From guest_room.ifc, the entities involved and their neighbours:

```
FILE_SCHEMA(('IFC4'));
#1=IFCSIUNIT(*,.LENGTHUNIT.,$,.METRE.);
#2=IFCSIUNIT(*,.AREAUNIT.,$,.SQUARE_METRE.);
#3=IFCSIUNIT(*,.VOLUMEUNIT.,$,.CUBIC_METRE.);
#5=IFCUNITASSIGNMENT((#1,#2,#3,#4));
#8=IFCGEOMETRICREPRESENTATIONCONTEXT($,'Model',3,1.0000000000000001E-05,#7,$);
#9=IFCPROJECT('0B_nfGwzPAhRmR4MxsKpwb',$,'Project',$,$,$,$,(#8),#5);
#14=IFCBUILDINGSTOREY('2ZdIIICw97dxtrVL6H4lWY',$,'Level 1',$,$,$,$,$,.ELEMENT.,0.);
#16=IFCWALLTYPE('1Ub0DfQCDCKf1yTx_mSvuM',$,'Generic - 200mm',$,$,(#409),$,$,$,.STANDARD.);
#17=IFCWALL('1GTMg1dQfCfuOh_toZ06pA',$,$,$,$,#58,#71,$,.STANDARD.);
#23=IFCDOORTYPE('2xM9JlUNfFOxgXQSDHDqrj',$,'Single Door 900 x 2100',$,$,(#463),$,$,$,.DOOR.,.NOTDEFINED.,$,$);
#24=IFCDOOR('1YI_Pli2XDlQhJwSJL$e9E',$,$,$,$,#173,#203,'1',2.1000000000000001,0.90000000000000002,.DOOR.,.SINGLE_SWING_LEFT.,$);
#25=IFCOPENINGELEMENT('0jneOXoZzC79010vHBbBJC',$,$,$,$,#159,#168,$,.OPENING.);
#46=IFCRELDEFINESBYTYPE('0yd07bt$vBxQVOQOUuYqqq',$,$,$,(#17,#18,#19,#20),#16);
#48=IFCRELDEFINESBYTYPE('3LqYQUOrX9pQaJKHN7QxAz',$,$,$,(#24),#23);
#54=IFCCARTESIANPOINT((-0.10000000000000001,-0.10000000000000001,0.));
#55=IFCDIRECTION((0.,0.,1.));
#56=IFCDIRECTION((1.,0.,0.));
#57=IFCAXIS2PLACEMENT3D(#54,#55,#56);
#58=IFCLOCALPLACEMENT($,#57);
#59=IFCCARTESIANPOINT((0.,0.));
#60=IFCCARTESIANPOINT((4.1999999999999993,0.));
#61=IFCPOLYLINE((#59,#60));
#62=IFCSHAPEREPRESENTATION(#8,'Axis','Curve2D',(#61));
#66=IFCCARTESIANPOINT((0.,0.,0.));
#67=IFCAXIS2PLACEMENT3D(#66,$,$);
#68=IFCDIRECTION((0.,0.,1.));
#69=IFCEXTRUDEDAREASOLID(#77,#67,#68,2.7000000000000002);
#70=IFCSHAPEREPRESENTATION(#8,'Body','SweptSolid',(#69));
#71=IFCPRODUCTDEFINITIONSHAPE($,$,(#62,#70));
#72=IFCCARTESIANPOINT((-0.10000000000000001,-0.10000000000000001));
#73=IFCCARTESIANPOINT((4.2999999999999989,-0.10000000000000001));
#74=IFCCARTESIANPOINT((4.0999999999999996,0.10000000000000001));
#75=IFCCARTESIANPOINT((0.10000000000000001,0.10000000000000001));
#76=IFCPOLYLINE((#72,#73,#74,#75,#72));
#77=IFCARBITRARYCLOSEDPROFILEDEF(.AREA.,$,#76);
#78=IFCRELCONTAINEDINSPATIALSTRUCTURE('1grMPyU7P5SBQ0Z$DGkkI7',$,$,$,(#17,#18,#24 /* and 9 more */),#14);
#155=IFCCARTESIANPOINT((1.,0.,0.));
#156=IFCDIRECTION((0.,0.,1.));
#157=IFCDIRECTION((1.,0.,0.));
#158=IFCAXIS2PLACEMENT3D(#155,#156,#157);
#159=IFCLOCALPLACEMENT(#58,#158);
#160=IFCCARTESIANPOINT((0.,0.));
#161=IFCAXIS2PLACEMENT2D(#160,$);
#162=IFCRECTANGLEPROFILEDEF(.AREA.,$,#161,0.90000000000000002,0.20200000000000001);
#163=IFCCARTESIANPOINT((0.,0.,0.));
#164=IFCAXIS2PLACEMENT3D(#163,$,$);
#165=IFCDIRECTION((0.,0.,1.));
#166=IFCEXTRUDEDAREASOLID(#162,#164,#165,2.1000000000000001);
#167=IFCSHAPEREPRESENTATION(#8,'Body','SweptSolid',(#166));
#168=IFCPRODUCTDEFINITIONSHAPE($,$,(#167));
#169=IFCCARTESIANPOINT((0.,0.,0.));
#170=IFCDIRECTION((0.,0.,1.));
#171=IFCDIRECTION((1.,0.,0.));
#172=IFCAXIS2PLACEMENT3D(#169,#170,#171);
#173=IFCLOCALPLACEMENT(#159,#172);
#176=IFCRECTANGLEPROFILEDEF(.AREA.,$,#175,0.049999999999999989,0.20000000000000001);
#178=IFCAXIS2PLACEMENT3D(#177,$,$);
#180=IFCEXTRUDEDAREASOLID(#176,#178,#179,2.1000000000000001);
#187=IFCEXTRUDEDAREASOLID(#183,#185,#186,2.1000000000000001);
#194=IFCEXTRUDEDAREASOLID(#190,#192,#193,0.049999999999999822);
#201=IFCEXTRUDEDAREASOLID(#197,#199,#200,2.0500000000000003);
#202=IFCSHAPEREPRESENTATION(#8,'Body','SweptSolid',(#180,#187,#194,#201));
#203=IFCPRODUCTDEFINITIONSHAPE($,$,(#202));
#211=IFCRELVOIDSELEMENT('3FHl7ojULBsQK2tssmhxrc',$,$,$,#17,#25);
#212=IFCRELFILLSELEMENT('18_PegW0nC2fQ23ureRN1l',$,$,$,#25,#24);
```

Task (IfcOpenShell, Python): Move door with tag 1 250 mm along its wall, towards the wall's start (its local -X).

```python
import ifcopenshell
import ifcopenshell.api.geometry
import ifcopenshell.util.placement
import ifcopenshell.util.unit

model = ifcopenshell.open("guest_room.ifc")
unit_scale = ifcopenshell.util.unit.calculate_unit_scale(model)

door = model.by_guid("1YI_Pli2XDlQhJwSJL$e9E")
opening = door.FillsVoids[0].RelatingOpeningElement
wall = opening.VoidsElements[0].RelatingBuildingElement

wall_matrix = ifcopenshell.util.placement.get_local_placement(wall.ObjectPlacement)
shift = wall_matrix[:3, 0] * -0.25 / unit_scale
before = ifcopenshell.util.placement.get_local_placement(door.ObjectPlacement)[:3, 3].copy()

# The door is placed relative to its opening, so it follows when the opening moves.
matrix = ifcopenshell.util.placement.get_local_placement(opening.ObjectPlacement)
matrix[:3, 3] += shift
ifcopenshell.api.geometry.edit_object_placement(
    model, product=opening, matrix=matrix, is_si=False, should_transform_children=True
)

after = ifcopenshell.util.placement.get_local_placement(door.ObjectPlacement)[:3, 3]
print("door moved by", (after - before).round(3) + 0.0)

model.write("guest_room_updated.ifc")
```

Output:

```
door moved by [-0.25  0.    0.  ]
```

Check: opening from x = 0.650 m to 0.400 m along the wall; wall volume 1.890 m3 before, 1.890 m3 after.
